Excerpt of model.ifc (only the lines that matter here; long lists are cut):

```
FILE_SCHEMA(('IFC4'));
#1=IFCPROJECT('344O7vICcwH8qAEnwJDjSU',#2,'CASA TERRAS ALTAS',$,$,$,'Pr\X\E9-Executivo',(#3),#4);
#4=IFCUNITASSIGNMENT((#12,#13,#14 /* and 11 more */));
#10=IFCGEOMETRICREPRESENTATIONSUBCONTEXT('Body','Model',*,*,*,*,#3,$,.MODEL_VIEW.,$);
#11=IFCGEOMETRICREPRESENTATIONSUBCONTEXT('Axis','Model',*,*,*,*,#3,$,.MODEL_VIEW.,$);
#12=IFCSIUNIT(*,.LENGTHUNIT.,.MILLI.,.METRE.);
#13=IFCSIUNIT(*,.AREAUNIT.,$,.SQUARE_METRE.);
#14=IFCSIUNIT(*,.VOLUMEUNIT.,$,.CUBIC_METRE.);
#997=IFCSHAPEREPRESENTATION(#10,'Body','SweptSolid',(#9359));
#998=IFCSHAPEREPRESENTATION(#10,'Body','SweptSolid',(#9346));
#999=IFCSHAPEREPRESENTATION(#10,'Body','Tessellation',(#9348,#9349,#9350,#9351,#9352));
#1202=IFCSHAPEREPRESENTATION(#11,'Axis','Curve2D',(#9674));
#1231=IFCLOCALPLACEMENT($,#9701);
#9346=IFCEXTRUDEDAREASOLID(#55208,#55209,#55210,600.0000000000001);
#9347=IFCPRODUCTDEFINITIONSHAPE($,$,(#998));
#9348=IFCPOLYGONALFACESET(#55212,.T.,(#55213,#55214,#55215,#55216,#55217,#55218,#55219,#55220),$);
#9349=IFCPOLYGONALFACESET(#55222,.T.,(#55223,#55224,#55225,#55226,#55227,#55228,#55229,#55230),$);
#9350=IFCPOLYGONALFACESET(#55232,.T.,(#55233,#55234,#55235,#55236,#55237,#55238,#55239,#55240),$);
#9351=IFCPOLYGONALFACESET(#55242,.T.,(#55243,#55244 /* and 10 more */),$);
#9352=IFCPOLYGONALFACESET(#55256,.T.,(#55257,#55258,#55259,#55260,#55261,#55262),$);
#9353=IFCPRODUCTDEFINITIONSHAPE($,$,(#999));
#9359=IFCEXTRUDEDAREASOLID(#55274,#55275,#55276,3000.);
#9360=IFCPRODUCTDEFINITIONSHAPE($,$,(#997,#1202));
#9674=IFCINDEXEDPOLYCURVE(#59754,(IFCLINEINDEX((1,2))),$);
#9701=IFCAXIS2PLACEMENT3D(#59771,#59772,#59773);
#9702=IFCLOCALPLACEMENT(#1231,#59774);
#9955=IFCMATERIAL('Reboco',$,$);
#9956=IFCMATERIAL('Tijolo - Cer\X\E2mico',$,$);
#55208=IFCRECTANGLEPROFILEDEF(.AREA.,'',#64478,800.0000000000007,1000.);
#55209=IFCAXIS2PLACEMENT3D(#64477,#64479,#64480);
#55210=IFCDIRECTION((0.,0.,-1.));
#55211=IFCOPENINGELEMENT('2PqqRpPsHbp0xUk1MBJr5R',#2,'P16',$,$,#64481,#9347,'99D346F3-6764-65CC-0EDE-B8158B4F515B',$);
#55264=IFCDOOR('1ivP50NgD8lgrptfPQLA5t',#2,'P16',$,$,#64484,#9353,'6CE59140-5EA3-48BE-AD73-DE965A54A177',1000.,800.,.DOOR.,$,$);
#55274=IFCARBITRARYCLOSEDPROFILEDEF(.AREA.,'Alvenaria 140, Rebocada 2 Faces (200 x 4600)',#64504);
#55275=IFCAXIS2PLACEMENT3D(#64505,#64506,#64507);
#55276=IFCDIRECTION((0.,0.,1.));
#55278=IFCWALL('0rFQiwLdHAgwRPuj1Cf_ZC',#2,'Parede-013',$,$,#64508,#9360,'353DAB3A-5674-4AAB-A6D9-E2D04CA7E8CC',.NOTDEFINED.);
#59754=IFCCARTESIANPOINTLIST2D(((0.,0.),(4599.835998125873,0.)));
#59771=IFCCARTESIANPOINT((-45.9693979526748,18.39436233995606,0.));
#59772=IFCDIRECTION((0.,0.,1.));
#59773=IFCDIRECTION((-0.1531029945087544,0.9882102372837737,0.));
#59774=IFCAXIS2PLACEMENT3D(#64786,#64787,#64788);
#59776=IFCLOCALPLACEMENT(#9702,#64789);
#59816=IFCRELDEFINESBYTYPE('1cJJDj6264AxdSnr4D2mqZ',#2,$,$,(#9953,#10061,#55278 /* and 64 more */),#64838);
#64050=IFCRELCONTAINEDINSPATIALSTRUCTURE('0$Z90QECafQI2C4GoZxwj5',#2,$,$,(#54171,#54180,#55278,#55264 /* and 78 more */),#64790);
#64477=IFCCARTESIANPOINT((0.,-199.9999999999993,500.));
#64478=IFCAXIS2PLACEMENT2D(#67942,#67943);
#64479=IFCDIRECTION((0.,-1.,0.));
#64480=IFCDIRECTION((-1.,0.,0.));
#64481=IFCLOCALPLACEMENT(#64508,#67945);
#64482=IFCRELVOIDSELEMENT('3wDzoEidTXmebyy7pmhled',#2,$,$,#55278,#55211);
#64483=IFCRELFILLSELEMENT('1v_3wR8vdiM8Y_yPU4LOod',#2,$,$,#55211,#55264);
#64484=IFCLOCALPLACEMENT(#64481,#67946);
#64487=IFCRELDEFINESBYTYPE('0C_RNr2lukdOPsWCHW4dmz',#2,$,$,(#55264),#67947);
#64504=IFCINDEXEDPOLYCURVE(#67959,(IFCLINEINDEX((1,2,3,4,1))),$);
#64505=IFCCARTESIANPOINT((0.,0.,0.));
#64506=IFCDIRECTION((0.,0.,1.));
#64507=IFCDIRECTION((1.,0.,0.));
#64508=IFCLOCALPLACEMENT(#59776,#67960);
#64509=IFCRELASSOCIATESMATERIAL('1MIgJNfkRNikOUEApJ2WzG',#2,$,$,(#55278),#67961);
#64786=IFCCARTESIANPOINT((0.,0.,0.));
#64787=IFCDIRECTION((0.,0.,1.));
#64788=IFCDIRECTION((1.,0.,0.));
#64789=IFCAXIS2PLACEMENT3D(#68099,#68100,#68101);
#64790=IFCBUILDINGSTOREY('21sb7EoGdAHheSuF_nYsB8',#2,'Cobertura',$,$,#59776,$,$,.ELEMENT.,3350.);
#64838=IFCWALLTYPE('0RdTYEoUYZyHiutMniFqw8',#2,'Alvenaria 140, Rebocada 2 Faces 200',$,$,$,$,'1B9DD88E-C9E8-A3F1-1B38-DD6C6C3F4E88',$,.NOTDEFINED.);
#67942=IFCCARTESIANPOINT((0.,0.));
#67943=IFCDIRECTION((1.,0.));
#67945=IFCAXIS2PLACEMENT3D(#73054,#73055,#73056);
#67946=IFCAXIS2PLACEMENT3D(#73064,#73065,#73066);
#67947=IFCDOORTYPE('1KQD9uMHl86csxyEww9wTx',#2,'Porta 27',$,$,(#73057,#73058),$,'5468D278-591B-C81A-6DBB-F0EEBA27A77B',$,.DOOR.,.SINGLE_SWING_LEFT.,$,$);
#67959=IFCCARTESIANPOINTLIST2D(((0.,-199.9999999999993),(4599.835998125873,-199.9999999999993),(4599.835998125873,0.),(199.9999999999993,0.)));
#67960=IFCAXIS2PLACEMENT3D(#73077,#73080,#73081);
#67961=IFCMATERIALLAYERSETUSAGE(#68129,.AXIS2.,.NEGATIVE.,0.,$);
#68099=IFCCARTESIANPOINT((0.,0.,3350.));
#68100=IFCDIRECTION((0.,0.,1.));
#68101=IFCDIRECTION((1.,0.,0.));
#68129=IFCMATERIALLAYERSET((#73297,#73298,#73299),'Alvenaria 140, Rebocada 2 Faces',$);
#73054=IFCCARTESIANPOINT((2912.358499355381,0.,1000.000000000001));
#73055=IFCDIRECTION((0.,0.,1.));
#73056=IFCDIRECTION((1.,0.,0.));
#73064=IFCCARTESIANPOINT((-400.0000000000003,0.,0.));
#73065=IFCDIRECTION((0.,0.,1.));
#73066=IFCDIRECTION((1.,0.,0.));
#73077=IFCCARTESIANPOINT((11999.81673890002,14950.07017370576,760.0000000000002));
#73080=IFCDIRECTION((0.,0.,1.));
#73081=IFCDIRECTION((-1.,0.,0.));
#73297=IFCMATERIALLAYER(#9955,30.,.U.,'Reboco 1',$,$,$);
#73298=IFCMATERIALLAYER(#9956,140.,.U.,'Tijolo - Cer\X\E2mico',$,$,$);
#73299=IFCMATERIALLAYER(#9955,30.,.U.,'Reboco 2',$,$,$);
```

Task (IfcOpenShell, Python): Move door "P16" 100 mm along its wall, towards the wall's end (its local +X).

```python
import ifcopenshell
import ifcopenshell.api.geometry
import ifcopenshell.util.placement
import ifcopenshell.util.unit

model = ifcopenshell.open("model.ifc")
unit_scale = ifcopenshell.util.unit.calculate_unit_scale(model)

door = model.by_id(55264)
opening = door.FillsVoids[0].RelatingOpeningElement
wall = opening.VoidsElements[0].RelatingBuildingElement

wall_matrix = ifcopenshell.util.placement.get_local_placement(wall.ObjectPlacement)
shift = wall_matrix[:3, 0] * 0.1 / unit_scale
before = ifcopenshell.util.placement.get_local_placement(door.ObjectPlacement)[:3, 3].copy()

# The door is placed relative to its opening, so it follows when the opening moves.
matrix = ifcopenshell.util.placement.get_local_placement(opening.ObjectPlacement)
matrix[:3, 3] += shift
ifcopenshell.api.geometry.edit_object_placement(
    model, product=opening, matrix=matrix, is_si=False, should_transform_children=True
)

after = ifcopenshell.util.placement.get_local_placement(door.ObjectPlacement)[:3, 3]
print("door moved by", (after - before).round(3) + 0.0)

model.write("model_v2.ifc")
```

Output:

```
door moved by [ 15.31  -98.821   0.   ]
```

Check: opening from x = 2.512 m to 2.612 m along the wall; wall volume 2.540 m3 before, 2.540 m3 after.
